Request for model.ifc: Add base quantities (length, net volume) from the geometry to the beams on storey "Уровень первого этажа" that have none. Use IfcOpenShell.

First a look at what the model holds.

```python
import ifcopenshell
import ifcopenshell.util.element
import ifcopenshell.util.unit

model = ifcopenshell.open("model.ifc")
print(model.schema)
for unit_type in ("LENGTHUNIT", "AREAUNIT", "VOLUMEUNIT"):
    print(unit_type, ifcopenshell.util.unit.calculate_unit_scale(model, unit_type))
storey = next(s for s in model.by_type("IfcBuildingStorey") if s.Name == "Уровень первого этажа")
beams = [e for e in ifcopenshell.util.element.get_decomposition(storey) if e.is_a("IfcBeam")]
for e in sorted(beams, key=lambda e: e.id()):
    print(e.id(), e.is_a(), e.Name, list(ifcopenshell.util.element.get_psets(e, qtos_only=True)), sep=" | ")
```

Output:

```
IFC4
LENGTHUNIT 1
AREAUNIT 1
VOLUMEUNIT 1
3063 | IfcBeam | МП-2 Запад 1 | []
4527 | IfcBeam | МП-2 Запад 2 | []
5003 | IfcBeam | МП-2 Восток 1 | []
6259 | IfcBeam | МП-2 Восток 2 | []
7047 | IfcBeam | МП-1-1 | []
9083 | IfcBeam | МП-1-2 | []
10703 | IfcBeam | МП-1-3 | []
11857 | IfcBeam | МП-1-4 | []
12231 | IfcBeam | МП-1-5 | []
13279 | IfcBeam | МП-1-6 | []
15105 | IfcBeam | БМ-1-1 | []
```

```python
import ifcopenshell
import ifcopenshell.api.pset
import ifcopenshell.geom
import ifcopenshell.util.element
import ifcopenshell.util.shape
import ifcopenshell.util.unit

model = ifcopenshell.open("model.ifc")
unit_scale = ifcopenshell.util.unit.calculate_unit_scale(model)
volume_scale = ifcopenshell.util.unit.calculate_unit_scale(model, "VOLUMEUNIT")
settings = ifcopenshell.geom.settings()

storey = next(s for s in model.by_type("IfcBuildingStorey") if s.Name == "Уровень первого этажа")
beams = [e for e in ifcopenshell.util.element.get_decomposition(storey) if e.is_a("IfcBeam")]

for e in sorted(beams, key=lambda e: e.id()):
    if ifcopenshell.util.element.get_psets(e, qtos_only=True, should_inherit=False):
        continue
    # Geometry comes back in metres, in the element's own axes.
    shape = ifcopenshell.geom.create_shape(settings, e)
    values = {
        "Length": ifcopenshell.util.shape.get_max_xyz(shape.geometry) / unit_scale,
        "NetVolume": ifcopenshell.util.shape.get_volume(shape.geometry) / volume_scale,
    }
    qto = ifcopenshell.api.pset.add_qto(model, product=e, name="Qto_BeamBaseQuantities")
    ifcopenshell.api.pset.edit_qto(model, qto=qto, properties=values)
    print(e.id(), {k: round(v, 3) for k, v in values.items()})

model.write("model-out.ifc")
```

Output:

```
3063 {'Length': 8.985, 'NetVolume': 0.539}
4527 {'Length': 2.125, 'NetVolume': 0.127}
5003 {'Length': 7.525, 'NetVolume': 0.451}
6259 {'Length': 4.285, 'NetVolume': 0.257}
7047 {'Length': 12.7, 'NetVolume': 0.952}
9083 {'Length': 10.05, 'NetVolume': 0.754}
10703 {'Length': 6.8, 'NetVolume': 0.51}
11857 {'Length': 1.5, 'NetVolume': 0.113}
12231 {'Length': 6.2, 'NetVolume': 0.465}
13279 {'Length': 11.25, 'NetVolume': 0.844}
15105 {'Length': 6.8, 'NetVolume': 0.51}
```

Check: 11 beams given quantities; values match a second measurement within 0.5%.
